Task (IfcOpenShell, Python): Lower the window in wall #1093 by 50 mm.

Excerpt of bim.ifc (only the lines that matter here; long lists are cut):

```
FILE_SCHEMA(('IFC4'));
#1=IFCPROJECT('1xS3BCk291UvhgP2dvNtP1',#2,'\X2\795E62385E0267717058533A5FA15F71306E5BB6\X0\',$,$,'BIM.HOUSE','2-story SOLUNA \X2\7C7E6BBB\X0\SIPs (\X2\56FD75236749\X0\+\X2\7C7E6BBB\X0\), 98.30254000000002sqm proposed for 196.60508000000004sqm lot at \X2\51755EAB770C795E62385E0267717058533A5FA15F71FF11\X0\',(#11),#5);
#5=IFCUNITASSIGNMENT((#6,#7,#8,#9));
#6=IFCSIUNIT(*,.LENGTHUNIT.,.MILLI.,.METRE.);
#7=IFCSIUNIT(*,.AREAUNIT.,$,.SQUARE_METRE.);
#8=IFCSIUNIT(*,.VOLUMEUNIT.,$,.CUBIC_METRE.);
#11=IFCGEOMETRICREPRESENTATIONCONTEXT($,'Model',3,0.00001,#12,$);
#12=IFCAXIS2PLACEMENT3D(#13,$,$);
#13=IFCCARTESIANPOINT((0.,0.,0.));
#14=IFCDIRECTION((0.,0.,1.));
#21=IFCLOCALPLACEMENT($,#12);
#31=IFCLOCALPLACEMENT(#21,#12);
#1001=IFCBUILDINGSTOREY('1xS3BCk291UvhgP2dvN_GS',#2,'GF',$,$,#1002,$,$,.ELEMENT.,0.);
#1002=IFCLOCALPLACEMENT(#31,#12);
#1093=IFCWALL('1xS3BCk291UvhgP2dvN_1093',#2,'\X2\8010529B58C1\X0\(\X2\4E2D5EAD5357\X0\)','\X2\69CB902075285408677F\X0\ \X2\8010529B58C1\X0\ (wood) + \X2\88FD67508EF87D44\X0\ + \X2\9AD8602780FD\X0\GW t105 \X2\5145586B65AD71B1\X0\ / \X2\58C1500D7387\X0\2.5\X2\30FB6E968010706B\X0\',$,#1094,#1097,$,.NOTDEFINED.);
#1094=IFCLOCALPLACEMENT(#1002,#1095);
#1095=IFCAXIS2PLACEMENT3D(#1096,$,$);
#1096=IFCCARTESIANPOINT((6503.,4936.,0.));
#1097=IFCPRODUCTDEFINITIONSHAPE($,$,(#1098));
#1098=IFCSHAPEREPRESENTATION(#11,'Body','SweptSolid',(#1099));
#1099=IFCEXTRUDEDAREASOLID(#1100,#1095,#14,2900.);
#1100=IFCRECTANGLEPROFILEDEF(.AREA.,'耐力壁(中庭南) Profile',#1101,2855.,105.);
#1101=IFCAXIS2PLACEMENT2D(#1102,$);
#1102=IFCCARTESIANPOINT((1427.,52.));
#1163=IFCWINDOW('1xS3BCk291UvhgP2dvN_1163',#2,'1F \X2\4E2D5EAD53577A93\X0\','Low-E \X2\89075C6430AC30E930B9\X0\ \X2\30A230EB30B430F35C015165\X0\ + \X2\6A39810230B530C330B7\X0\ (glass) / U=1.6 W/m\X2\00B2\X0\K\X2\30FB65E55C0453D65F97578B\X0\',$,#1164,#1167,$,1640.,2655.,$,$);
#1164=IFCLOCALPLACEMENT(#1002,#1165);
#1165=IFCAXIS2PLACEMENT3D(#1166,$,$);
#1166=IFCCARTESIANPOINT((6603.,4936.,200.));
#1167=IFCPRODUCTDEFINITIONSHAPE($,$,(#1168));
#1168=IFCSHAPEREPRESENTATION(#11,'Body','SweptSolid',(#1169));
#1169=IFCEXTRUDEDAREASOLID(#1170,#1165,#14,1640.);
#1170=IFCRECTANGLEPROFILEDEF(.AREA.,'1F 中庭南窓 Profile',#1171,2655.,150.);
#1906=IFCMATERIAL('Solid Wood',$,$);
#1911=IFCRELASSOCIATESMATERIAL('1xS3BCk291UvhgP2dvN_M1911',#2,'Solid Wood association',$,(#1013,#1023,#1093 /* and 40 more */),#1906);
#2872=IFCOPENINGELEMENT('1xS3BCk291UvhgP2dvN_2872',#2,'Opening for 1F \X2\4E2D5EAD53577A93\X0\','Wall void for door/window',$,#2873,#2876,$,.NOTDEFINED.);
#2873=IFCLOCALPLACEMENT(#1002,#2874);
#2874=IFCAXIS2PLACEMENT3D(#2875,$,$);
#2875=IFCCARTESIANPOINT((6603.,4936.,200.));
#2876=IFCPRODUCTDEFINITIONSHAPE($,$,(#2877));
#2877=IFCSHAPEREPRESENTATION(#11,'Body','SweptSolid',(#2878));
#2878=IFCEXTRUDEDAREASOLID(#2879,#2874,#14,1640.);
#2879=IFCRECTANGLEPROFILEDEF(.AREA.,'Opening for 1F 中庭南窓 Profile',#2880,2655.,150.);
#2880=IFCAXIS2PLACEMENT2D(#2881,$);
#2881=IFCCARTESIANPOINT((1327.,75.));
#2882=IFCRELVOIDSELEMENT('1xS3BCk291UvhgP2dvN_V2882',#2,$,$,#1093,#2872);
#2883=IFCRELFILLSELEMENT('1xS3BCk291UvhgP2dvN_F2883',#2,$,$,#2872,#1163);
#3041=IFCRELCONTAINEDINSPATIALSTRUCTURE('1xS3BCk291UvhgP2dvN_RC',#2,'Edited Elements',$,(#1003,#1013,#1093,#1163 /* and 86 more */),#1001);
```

```python
import numpy as np
import ifcopenshell
import ifcopenshell.api.geometry
import ifcopenshell.util.placement
import ifcopenshell.util.unit

model = ifcopenshell.open("bim.ifc")
unit_scale = ifcopenshell.util.unit.calculate_unit_scale(model)

window = model.by_id(1163)
opening = window.FillsVoids[0].RelatingOpeningElement
dz = -0.05 / unit_scale

shift = np.array([0.0, 0.0, dz])
# The window is not placed relative to its opening, so move both.
for product in (opening, window):
    matrix = ifcopenshell.util.placement.get_local_placement(product.ObjectPlacement)
    matrix[:3, 3] += shift
    ifcopenshell.api.geometry.edit_object_placement(model, product=product, matrix=matrix, is_si=False)

print(f"moved by {dz * unit_scale:+.3f} m")

model.write("bim_updated.ifc")
```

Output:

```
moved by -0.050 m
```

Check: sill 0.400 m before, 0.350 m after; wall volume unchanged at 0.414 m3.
